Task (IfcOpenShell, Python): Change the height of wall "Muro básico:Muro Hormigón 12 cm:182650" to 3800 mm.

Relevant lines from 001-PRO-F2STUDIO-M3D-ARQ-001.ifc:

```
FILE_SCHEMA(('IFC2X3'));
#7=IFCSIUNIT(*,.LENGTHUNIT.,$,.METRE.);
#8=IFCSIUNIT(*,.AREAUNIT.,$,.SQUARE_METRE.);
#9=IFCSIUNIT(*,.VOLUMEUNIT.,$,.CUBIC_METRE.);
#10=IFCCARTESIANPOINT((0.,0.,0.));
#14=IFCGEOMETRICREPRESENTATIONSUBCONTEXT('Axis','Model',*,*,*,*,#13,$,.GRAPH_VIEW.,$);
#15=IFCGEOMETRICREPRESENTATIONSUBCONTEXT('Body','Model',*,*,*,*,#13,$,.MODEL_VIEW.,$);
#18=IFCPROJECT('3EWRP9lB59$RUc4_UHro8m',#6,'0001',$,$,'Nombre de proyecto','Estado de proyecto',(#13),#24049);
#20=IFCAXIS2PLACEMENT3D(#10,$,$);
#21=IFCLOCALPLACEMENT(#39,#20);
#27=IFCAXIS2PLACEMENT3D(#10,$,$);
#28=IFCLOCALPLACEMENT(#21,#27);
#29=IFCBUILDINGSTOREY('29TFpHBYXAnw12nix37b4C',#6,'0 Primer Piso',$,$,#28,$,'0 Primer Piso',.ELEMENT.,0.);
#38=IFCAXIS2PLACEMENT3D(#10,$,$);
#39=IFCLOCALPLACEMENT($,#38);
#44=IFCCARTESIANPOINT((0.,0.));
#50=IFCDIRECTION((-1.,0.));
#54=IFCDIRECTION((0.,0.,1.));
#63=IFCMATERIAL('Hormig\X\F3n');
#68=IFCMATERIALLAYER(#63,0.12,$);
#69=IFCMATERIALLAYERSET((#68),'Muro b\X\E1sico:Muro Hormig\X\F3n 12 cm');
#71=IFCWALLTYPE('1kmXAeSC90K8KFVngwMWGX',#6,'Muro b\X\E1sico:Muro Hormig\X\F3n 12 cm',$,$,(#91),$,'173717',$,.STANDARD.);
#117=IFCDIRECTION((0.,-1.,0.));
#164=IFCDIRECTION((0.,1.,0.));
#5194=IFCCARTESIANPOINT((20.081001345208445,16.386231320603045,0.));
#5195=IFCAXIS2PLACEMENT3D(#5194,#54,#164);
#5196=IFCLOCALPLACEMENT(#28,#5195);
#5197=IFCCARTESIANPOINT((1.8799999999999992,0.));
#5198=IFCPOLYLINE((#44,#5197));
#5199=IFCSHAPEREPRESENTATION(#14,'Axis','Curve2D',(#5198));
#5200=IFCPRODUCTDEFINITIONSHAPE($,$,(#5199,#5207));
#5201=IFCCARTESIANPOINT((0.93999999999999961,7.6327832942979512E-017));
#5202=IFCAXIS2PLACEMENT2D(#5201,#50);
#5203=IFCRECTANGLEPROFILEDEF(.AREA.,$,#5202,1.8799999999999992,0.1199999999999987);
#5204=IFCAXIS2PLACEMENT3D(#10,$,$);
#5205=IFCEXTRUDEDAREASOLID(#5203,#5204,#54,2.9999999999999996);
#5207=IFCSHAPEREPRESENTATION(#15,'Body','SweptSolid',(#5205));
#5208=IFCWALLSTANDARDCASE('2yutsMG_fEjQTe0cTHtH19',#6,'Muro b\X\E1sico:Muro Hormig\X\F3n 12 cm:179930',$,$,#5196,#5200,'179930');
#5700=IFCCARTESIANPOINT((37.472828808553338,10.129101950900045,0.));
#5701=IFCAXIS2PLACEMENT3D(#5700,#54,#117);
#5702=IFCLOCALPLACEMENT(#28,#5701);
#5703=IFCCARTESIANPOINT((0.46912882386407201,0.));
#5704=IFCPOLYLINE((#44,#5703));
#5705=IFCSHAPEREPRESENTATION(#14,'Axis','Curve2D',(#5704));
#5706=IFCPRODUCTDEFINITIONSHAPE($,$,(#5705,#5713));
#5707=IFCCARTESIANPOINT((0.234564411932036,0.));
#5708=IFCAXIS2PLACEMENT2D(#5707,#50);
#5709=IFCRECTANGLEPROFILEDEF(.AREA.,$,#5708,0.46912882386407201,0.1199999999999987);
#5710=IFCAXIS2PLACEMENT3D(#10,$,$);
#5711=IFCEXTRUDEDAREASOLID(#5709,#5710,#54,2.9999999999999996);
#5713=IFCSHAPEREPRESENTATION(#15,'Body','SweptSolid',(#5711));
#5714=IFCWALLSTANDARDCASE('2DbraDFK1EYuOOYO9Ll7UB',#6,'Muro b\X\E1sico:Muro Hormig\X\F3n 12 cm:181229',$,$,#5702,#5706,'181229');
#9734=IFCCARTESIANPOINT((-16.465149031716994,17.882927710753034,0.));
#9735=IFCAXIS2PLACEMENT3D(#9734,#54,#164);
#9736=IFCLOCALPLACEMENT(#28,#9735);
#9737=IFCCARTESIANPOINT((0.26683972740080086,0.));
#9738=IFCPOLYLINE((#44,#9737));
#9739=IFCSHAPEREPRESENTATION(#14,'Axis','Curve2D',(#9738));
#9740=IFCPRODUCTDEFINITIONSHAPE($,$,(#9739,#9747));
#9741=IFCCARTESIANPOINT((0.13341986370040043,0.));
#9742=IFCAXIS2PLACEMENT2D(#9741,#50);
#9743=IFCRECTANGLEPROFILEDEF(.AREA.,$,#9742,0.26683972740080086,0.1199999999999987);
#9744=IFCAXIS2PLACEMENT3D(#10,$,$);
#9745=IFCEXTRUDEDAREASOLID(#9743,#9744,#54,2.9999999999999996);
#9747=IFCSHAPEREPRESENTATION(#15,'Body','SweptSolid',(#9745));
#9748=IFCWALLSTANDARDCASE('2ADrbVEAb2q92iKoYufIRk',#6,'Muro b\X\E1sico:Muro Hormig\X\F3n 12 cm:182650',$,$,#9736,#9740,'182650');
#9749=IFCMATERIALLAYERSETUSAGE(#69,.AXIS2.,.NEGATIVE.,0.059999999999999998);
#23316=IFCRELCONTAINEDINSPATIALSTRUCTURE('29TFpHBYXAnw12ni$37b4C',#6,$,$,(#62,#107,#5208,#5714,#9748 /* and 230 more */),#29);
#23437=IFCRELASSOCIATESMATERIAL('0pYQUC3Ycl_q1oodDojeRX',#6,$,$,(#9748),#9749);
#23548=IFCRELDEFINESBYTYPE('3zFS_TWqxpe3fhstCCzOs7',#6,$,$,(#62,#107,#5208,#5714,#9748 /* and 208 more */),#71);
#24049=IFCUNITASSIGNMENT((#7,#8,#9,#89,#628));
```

```python
import ifcopenshell
import ifcopenshell.geom
import ifcopenshell.util.representation
import ifcopenshell.util.shape
import ifcopenshell.util.unit

model = ifcopenshell.open("001-PRO-F2STUDIO-M3D-ARQ-001.ifc")
unit_scale = ifcopenshell.util.unit.calculate_unit_scale(model)
settings = ifcopenshell.geom.settings()


def volume(element):
    """Net volume in cubic metres, openings subtracted."""
    shape = ifcopenshell.geom.create_shape(settings, element)
    return ifcopenshell.util.shape.get_volume(shape.geometry)


wall = model.by_guid("2ADrbVEAb2q92iKoYufIRk")
before = volume(wall)

body = ifcopenshell.util.representation.get_representation(wall, "Model", "Body")
solid = body.Items[0]
old_height = solid.Depth
solid.Depth = 3.8 / unit_scale
after = volume(wall)

print(f"height {old_height:g} -> {solid.Depth:g}, volume {before:.3f} -> {after:.3f} m3")

model.write("001-PRO-F2STUDIO-M3D-ARQ-001_v2.ifc")
```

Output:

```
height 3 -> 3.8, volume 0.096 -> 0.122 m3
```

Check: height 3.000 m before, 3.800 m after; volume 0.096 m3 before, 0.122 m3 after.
